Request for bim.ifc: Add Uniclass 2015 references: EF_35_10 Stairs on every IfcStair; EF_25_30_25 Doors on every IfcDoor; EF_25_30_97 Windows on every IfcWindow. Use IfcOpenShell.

First a look at what the model holds.

```python
import ifcopenshell

model = ifcopenshell.open("bim.ifc")
print(model.schema)
print("classifications:", [c.Name for c in model.by_type("IfcClassification")])
for ifc_class in ("IfcDoor", "IfcRoof", "IfcStair", "IfcWall", "IfcWindow"):
    print(ifc_class, len(model.by_type(ifc_class)))
```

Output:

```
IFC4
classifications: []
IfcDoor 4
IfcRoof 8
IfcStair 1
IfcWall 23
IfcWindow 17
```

```python
import ifcopenshell
import ifcopenshell.api.classification

model = ifcopenshell.open("bim.ifc")

system = ifcopenshell.api.classification.add_classification(model, classification="Uniclass 2015")

codes = {
    "IfcStair": ("EF_35_10", "Stairs"),
    "IfcDoor": ("EF_25_30_25", "Doors"),
    "IfcWindow": ("EF_25_30_97", "Windows"),
}
for ifc_class, (code, name) in codes.items():
    products = model.by_type(ifc_class)
    ifcopenshell.api.classification.add_reference(
        model, products=products, classification=system, identification=code, name=name
    )
    print(code, len(products))

model.write("bim_rev.ifc")
```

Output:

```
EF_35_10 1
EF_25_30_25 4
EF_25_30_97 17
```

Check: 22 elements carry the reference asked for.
